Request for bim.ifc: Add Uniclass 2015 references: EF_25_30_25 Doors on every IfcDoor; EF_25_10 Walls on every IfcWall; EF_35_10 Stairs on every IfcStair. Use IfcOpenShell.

First a look at what the model holds.

```python
import ifcopenshell

model = ifcopenshell.open("bim.ifc")
print(model.schema)
print("classifications:", [c.Name for c in model.by_type("IfcClassification")])
for ifc_class in ("IfcDoor", "IfcRoof", "IfcStair", "IfcWall", "IfcWindow"):
    print(ifc_class, len(model.by_type(ifc_class)))
```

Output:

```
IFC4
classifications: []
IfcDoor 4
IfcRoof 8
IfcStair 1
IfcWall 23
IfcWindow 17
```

```python
import ifcopenshell
import ifcopenshell.api.classification

model = ifcopenshell.open("bim.ifc")

system = ifcopenshell.api.classification.add_classification(model, classification="Uniclass 2015")

codes = {
    "IfcDoor": ("EF_25_30_25", "Doors"),
    "IfcWall": ("EF_25_10", "Walls"),
    "IfcStair": ("EF_35_10", "Stairs"),
}
for ifc_class, (code, name) in codes.items():
    products = model.by_type(ifc_class)
    ifcopenshell.api.classification.add_reference(
        model, products=products, classification=system, identification=code, name=name
    )
    print(code, len(products))

model.write("bim-out.ifc")
```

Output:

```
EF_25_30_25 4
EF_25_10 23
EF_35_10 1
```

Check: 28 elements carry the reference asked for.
